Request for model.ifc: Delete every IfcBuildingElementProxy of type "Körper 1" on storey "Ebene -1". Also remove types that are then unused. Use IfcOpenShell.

First a look at what the model holds.

```python
import ifcopenshell
import ifcopenshell.util.element

model = ifcopenshell.open("model.ifc")
print(model.schema)
storey = next(s for s in model.by_type("IfcBuildingStorey") if s.Name == "Ebene -1")
proxies = [e for e in ifcopenshell.util.element.get_decomposition(storey) if e.is_a("IfcBuildingElementProxy")]
seen = {}
for e in proxies:
    element_type = ifcopenshell.util.element.get_type(e)
    name = element_type.Name if element_type not in (None, e) else None
    seen[name] = seen.get(name, 0) + 1
for name, count in sorted(seen.items(), key=str):
    print(count, "x", name)
```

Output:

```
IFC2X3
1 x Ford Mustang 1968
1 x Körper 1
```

```python
import ifcopenshell
import ifcopenshell.api.root
import ifcopenshell.util.element

model = ifcopenshell.open("model.ifc")

storey = next(s for s in model.by_type("IfcBuildingStorey") if s.Name == "Ebene -1")
proxies = [e for e in ifcopenshell.util.element.get_decomposition(storey) if e.is_a("IfcBuildingElementProxy")]
targets = [e for e in proxies if (t := ifcopenshell.util.element.get_type(e)) not in (None, e) and t.Name == "Körper 1"]
types = {ifcopenshell.util.element.get_type(e) for e in targets} - {None, *targets}

for e in targets:
    ifcopenshell.api.root.remove_product(model, product=e)
print(len(targets), "removed")

unused = [t for t in types if not ifcopenshell.util.element.get_types(t)]
for t in unused:
    ifcopenshell.api.root.remove_product(model, product=t)
print(len(unused), "unused types removed")

model.write("model_v2.ifc")
```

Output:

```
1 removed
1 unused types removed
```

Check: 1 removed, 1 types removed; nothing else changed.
